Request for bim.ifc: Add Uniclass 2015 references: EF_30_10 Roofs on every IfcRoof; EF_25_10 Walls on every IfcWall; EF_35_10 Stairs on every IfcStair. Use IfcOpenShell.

First a look at what the model holds.

```python
import ifcopenshell

model = ifcopenshell.open("bim.ifc")
print(model.schema)
print("classifications:", [c.Name for c in model.by_type("IfcClassification")])
for ifc_class in ("IfcDoor", "IfcRoof", "IfcStair", "IfcWall", "IfcWindow"):
    print(ifc_class, len(model.by_type(ifc_class)))
```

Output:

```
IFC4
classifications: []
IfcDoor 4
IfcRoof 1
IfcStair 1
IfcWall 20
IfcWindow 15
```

```python
import ifcopenshell
import ifcopenshell.api.classification

model = ifcopenshell.open("bim.ifc")

system = ifcopenshell.api.classification.add_classification(model, classification="Uniclass 2015")

codes = {
    "IfcRoof": ("EF_30_10", "Roofs"),
    "IfcWall": ("EF_25_10", "Walls"),
    "IfcStair": ("EF_35_10", "Stairs"),
}
for ifc_class, (code, name) in codes.items():
    products = model.by_type(ifc_class)
    ifcopenshell.api.classification.add_reference(
        model, products=products, classification=system, identification=code, name=name
    )
    print(code, len(products))

model.write("bim-out.ifc")
```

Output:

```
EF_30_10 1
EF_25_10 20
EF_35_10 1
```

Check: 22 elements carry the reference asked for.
